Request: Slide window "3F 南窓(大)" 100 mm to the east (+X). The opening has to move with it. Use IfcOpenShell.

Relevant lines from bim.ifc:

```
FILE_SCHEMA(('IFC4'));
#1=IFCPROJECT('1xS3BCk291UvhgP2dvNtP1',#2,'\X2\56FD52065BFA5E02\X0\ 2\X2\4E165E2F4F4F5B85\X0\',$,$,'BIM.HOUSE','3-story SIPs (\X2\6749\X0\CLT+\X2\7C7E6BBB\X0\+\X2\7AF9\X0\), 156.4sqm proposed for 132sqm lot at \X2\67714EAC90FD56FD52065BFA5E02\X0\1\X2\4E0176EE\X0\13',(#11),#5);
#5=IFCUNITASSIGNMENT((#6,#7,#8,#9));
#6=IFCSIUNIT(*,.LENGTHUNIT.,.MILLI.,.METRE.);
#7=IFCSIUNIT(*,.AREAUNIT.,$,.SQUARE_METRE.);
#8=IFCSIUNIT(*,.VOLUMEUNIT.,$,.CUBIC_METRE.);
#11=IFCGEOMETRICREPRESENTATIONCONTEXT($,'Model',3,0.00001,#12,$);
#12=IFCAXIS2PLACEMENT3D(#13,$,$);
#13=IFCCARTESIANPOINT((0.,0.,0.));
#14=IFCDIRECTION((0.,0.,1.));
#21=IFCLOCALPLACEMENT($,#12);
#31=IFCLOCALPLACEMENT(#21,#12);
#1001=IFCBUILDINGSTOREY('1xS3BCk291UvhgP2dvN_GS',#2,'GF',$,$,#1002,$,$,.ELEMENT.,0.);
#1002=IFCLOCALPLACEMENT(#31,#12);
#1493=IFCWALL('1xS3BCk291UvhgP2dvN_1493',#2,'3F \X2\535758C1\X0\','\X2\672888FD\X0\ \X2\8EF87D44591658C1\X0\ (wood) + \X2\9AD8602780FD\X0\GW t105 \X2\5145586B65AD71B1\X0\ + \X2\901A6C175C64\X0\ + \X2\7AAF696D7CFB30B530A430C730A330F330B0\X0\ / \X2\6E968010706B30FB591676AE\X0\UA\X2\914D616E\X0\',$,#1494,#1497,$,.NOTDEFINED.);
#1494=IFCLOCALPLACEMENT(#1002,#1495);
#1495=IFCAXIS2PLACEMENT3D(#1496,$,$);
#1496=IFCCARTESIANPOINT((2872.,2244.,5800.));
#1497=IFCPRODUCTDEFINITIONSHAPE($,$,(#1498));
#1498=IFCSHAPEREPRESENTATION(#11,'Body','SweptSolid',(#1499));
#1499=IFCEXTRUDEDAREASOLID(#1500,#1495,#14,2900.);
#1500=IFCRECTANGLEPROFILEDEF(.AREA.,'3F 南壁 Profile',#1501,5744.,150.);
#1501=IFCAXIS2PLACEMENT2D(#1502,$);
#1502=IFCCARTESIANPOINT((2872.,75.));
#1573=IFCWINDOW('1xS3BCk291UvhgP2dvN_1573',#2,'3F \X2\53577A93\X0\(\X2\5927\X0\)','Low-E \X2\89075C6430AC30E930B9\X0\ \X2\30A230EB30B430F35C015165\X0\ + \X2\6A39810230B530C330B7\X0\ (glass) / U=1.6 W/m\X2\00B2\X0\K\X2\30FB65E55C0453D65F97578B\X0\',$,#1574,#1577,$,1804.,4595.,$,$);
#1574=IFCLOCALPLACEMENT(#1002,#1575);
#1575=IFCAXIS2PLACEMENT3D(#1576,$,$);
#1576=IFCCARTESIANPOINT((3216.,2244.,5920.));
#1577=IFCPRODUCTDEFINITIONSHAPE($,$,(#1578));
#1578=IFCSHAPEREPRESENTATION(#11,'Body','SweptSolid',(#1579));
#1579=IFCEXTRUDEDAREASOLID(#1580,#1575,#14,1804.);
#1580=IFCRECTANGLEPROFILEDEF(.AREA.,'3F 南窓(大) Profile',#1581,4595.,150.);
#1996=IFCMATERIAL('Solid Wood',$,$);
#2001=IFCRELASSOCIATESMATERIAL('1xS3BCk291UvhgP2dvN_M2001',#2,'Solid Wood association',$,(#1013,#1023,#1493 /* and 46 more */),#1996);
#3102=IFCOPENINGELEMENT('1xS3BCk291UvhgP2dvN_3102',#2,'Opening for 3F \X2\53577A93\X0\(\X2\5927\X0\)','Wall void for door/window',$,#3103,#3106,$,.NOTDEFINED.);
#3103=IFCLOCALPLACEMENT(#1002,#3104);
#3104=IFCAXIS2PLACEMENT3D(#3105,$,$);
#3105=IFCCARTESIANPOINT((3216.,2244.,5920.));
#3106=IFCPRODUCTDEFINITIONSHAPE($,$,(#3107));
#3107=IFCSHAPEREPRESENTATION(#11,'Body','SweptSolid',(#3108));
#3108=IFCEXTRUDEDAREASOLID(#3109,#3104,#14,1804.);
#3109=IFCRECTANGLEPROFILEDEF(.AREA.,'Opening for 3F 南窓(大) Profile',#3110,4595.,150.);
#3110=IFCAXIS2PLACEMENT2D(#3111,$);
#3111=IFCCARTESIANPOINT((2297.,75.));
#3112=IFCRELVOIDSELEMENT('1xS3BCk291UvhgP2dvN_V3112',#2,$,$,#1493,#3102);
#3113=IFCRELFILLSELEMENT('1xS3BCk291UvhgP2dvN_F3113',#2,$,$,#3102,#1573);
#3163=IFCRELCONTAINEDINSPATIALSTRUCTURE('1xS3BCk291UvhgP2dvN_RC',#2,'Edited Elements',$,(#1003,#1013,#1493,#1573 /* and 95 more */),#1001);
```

```python
import ifcopenshell
import ifcopenshell.api.geometry
import ifcopenshell.util.placement

model = ifcopenshell.open("bim.ifc")

window = model.by_id(1573)
opening = window.FillsVoids[0].RelatingOpeningElement
wall = opening.VoidsElements[0].RelatingBuildingElement

wall_matrix = ifcopenshell.util.placement.get_local_placement(wall.ObjectPlacement)
shift = wall_matrix[:3, 0] * 100.0
before = ifcopenshell.util.placement.get_local_placement(window.ObjectPlacement)[:3, 3].copy()

# The window is not placed relative to its opening, so move both.
for product in (opening, window):
    matrix = ifcopenshell.util.placement.get_local_placement(product.ObjectPlacement)
    matrix[:3, 3] += shift
    ifcopenshell.api.geometry.edit_object_placement(model, product=product, matrix=matrix, is_si=False)

after = ifcopenshell.util.placement.get_local_placement(window.ObjectPlacement)[:3, 3]
print("window moved by", (after - before).round(3) + 0.0)

model.write("bim_rev.ifc")
```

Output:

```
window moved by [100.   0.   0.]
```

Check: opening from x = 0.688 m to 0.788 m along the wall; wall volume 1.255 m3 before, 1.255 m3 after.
